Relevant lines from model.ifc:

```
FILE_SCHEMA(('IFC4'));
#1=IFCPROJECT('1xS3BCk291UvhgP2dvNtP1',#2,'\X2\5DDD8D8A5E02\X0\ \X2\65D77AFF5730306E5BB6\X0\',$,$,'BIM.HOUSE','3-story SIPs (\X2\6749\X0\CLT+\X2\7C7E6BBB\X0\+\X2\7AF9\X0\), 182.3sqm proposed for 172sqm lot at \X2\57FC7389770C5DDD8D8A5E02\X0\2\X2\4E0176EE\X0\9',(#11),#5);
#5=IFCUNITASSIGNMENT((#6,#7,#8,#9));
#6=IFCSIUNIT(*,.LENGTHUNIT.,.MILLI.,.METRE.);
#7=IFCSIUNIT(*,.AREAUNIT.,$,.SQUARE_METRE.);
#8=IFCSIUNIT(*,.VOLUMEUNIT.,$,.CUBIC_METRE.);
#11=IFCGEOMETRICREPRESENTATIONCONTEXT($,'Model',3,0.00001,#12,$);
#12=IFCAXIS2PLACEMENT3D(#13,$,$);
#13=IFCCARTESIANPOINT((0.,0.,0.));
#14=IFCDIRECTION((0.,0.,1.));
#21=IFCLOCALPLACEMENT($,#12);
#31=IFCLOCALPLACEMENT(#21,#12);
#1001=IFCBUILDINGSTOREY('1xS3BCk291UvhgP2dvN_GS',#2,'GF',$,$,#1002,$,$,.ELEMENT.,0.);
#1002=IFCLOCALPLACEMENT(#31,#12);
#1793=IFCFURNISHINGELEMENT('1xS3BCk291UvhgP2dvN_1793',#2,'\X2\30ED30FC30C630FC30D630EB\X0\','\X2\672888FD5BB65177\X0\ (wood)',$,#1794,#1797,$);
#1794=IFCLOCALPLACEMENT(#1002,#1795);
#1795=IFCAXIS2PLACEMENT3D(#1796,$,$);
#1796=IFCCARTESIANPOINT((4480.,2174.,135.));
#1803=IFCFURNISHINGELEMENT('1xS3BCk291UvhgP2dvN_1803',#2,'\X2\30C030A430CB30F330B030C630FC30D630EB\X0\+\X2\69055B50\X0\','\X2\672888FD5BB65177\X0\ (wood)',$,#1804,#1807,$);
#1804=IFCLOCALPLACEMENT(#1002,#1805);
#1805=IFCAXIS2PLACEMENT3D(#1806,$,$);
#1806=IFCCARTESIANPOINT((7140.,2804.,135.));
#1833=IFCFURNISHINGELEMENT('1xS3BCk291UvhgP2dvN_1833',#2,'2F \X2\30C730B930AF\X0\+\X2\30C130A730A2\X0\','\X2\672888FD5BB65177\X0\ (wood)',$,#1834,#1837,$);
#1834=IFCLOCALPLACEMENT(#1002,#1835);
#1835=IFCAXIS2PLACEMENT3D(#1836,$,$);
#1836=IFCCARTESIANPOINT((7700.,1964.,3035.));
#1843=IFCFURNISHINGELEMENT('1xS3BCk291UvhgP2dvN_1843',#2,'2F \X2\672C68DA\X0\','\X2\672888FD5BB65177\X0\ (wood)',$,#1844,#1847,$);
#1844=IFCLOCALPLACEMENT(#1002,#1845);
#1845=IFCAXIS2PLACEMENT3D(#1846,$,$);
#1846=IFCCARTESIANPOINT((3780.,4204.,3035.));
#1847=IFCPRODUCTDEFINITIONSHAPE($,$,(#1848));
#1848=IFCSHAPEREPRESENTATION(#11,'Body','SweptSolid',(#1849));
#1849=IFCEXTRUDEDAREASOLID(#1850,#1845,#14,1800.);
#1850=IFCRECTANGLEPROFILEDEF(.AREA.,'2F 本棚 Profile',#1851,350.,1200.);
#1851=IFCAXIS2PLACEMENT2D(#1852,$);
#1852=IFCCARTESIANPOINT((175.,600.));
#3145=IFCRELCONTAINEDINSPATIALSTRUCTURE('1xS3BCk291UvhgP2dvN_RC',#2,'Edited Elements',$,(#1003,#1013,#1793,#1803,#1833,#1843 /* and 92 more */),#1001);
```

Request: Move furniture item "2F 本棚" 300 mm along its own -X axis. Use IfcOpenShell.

```python
import ifcopenshell
import ifcopenshell.api.geometry
import ifcopenshell.util.placement

model = ifcopenshell.open("model.ifc")

item = model.by_guid("1xS3BCk291UvhgP2dvN_1843")
matrix = ifcopenshell.util.placement.get_local_placement(item.ObjectPlacement)
matrix[:3, 3] -= matrix[:3, 0] * 300.0
ifcopenshell.api.geometry.edit_object_placement(model, product=item, matrix=matrix, is_si=False)

print(ifcopenshell.util.placement.get_local_placement(item.ObjectPlacement).round(3) + 0.0)

model.write("model-out.ifc")
```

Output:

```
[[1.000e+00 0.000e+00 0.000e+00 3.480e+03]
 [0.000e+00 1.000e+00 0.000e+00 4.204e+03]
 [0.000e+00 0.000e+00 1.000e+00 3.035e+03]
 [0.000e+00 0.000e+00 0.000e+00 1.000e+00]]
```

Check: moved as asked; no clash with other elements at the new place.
